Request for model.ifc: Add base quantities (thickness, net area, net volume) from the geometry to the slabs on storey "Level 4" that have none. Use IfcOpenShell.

First a look at what the model holds.

```python
import ifcopenshell
import ifcopenshell.util.element
import ifcopenshell.util.unit

model = ifcopenshell.open("model.ifc")
print(model.schema)
for unit_type in ("LENGTHUNIT", "AREAUNIT", "VOLUMEUNIT"):
    print(unit_type, ifcopenshell.util.unit.calculate_unit_scale(model, unit_type))
storey = next(s for s in model.by_type("IfcBuildingStorey") if s.Name == "Level 4")
slabs = [e for e in ifcopenshell.util.element.get_decomposition(storey) if e.is_a("IfcSlab")]
for e in sorted(slabs, key=lambda e: e.id()):
    print(e.id(), e.is_a(), e.Name, list(ifcopenshell.util.element.get_psets(e, qtos_only=True)), sep=" | ")
```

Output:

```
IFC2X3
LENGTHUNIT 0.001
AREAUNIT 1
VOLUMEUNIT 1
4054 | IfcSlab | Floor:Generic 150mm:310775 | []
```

```python
import ifcopenshell
import ifcopenshell.api.pset
import ifcopenshell.geom
import ifcopenshell.util.element
import ifcopenshell.util.shape
import ifcopenshell.util.unit

model = ifcopenshell.open("model.ifc")
unit_scale = ifcopenshell.util.unit.calculate_unit_scale(model)
area_scale = ifcopenshell.util.unit.calculate_unit_scale(model, "AREAUNIT")
volume_scale = ifcopenshell.util.unit.calculate_unit_scale(model, "VOLUMEUNIT")
settings = ifcopenshell.geom.settings()

storey = next(s for s in model.by_type("IfcBuildingStorey") if s.Name == "Level 4")
slabs = [e for e in ifcopenshell.util.element.get_decomposition(storey) if e.is_a("IfcSlab")]

for e in sorted(slabs, key=lambda e: e.id()):
    if ifcopenshell.util.element.get_psets(e, qtos_only=True, should_inherit=False):
        continue
    # Geometry comes back in metres, in the element's own axes.
    shape = ifcopenshell.geom.create_shape(settings, e)
    values = {
        "Width": ifcopenshell.util.shape.get_z(shape.geometry) / unit_scale,
        "NetArea": ifcopenshell.util.shape.get_footprint_area(shape.geometry) / area_scale,
        "NetVolume": ifcopenshell.util.shape.get_volume(shape.geometry) / volume_scale,
    }
    qto = ifcopenshell.api.pset.add_qto(model, product=e, name="BaseQuantities")
    ifcopenshell.api.pset.edit_qto(model, qto=qto, properties=values)
    print(e.id(), {k: round(v, 3) for k, v in values.items()})

model.write("model_v2.ifc")
```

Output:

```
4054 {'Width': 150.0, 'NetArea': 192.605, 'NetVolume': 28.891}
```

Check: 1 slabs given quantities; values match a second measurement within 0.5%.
